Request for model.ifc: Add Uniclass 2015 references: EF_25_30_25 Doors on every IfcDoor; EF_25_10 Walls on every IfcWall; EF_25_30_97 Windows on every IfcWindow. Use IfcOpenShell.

First a look at what the model holds.

```python
import ifcopenshell

model = ifcopenshell.open("model.ifc")
print(model.schema)
print("classifications:", [c.Name for c in model.by_type("IfcClassification")])
for ifc_class in ("IfcDoor", "IfcRoof", "IfcStair", "IfcWall", "IfcWindow"):
    print(ifc_class, len(model.by_type(ifc_class)))
```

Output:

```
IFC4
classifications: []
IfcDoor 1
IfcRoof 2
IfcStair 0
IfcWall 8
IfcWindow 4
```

```python
import ifcopenshell
import ifcopenshell.api.classification

model = ifcopenshell.open("model.ifc")

system = ifcopenshell.api.classification.add_classification(model, classification="Uniclass 2015")

codes = {
    "IfcDoor": ("EF_25_30_25", "Doors"),
    "IfcWall": ("EF_25_10", "Walls"),
    "IfcWindow": ("EF_25_30_97", "Windows"),
}
for ifc_class, (code, name) in codes.items():
    products = model.by_type(ifc_class)
    ifcopenshell.api.classification.add_reference(
        model, products=products, classification=system, identification=code, name=name
    )
    print(code, len(products))

model.write("model_updated.ifc")
```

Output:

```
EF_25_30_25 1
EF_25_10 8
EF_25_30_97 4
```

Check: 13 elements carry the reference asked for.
